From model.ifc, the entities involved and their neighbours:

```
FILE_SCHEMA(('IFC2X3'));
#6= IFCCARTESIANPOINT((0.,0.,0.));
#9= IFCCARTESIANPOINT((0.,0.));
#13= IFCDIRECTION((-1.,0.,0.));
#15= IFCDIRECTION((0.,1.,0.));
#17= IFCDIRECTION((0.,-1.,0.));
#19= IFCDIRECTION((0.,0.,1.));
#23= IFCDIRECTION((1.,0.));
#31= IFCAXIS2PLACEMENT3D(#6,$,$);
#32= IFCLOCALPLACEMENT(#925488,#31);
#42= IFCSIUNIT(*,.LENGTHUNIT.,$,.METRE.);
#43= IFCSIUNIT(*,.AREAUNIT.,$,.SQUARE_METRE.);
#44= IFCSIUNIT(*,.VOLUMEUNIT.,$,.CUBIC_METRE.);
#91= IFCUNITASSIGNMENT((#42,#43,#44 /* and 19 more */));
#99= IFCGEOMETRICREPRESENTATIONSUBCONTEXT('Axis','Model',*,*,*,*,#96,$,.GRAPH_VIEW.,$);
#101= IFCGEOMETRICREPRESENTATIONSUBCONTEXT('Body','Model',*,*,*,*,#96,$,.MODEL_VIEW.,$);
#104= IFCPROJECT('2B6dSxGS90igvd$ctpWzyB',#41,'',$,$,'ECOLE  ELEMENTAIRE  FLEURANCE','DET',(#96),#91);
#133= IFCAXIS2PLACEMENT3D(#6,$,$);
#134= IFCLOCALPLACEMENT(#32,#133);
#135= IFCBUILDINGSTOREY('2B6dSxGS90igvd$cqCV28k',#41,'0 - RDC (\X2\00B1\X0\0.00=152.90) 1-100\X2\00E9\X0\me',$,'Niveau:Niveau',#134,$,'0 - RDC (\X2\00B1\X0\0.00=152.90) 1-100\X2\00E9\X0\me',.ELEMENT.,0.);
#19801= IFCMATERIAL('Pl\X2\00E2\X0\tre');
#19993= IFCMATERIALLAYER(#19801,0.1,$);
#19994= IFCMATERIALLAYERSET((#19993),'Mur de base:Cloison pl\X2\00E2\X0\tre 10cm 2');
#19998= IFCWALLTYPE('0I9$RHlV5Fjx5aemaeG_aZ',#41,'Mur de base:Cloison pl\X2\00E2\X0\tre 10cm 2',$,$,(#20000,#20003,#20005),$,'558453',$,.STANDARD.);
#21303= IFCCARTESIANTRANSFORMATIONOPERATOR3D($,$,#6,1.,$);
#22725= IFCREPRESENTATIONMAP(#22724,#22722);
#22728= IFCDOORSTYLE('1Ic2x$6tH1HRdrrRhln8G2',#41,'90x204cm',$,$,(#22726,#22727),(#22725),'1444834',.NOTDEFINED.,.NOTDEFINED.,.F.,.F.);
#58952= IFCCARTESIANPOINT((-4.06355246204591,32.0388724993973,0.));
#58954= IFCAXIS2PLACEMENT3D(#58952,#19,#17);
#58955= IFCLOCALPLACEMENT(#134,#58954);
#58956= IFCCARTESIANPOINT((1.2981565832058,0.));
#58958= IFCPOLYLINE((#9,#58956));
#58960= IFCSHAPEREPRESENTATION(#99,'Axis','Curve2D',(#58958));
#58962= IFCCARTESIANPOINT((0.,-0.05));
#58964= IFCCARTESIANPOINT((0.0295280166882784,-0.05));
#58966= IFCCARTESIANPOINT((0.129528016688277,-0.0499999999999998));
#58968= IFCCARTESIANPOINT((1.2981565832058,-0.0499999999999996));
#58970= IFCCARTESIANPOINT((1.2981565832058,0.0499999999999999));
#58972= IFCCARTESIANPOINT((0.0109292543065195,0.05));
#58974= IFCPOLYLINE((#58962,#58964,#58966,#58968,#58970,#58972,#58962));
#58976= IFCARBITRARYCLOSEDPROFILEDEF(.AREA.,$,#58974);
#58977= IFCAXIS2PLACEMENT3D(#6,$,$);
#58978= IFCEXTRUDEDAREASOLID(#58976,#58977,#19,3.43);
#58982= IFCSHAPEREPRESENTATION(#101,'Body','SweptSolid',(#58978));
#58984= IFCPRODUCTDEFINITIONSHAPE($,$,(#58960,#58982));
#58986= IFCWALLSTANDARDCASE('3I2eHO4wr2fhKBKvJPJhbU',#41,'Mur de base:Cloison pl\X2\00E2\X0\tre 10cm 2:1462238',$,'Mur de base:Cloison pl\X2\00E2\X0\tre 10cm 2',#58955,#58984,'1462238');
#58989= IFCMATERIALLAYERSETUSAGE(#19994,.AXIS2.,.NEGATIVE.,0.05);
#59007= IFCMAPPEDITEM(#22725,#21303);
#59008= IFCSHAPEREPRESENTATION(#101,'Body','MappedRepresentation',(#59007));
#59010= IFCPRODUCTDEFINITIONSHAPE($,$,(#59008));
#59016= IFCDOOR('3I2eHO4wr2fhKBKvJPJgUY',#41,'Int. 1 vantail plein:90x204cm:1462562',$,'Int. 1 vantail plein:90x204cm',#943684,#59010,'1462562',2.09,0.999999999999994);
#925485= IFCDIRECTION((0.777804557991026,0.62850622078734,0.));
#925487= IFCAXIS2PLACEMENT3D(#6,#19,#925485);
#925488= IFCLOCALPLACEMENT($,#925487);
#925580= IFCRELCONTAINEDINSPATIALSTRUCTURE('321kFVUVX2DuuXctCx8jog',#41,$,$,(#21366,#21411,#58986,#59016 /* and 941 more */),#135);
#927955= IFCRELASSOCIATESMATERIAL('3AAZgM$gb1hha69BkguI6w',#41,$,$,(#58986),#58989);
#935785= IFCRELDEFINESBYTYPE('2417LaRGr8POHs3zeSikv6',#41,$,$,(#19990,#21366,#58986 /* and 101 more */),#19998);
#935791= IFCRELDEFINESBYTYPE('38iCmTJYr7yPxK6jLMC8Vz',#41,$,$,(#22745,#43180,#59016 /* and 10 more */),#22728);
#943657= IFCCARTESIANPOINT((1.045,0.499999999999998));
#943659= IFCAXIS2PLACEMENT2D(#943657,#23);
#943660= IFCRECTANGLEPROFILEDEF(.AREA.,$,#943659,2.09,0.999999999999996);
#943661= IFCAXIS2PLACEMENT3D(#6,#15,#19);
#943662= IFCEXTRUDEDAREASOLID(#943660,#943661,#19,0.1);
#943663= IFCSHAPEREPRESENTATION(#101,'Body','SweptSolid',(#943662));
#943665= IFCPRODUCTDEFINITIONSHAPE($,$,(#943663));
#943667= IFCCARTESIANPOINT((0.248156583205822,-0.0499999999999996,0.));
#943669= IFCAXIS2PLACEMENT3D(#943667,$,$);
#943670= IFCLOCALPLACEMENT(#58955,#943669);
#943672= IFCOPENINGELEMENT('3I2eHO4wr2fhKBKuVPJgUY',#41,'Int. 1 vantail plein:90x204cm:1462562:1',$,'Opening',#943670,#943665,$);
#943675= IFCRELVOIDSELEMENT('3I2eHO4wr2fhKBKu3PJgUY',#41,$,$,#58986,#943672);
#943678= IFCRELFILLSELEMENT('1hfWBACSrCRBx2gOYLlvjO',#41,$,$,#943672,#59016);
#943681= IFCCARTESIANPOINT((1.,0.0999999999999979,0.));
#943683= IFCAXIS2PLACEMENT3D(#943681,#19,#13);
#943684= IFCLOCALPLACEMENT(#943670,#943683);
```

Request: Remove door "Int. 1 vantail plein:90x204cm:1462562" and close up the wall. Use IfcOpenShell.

```python
import ifcopenshell
import ifcopenshell.api.feature
import ifcopenshell.api.root
import ifcopenshell.geom
import ifcopenshell.util.shape

model = ifcopenshell.open("model.ifc")
settings = ifcopenshell.geom.settings()


def volume(element):
    """Net volume in cubic metres, openings subtracted."""
    shape = ifcopenshell.geom.create_shape(settings, element)
    return ifcopenshell.util.shape.get_volume(shape.geometry)


door = model.by_id(59016)
opening = door.FillsVoids[0].RelatingOpeningElement
wall = opening.VoidsElements[0].RelatingBuildingElement
before = volume(wall)

ifcopenshell.api.root.remove_product(model, product=door)
ifcopenshell.api.feature.remove_feature(model, feature=opening)

after = volume(wall)

print(f"wall volume {before:.3f} -> {after:.3f} m3")

model.write("model_v2.ifc")
```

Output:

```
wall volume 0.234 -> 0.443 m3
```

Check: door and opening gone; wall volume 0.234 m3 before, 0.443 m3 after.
